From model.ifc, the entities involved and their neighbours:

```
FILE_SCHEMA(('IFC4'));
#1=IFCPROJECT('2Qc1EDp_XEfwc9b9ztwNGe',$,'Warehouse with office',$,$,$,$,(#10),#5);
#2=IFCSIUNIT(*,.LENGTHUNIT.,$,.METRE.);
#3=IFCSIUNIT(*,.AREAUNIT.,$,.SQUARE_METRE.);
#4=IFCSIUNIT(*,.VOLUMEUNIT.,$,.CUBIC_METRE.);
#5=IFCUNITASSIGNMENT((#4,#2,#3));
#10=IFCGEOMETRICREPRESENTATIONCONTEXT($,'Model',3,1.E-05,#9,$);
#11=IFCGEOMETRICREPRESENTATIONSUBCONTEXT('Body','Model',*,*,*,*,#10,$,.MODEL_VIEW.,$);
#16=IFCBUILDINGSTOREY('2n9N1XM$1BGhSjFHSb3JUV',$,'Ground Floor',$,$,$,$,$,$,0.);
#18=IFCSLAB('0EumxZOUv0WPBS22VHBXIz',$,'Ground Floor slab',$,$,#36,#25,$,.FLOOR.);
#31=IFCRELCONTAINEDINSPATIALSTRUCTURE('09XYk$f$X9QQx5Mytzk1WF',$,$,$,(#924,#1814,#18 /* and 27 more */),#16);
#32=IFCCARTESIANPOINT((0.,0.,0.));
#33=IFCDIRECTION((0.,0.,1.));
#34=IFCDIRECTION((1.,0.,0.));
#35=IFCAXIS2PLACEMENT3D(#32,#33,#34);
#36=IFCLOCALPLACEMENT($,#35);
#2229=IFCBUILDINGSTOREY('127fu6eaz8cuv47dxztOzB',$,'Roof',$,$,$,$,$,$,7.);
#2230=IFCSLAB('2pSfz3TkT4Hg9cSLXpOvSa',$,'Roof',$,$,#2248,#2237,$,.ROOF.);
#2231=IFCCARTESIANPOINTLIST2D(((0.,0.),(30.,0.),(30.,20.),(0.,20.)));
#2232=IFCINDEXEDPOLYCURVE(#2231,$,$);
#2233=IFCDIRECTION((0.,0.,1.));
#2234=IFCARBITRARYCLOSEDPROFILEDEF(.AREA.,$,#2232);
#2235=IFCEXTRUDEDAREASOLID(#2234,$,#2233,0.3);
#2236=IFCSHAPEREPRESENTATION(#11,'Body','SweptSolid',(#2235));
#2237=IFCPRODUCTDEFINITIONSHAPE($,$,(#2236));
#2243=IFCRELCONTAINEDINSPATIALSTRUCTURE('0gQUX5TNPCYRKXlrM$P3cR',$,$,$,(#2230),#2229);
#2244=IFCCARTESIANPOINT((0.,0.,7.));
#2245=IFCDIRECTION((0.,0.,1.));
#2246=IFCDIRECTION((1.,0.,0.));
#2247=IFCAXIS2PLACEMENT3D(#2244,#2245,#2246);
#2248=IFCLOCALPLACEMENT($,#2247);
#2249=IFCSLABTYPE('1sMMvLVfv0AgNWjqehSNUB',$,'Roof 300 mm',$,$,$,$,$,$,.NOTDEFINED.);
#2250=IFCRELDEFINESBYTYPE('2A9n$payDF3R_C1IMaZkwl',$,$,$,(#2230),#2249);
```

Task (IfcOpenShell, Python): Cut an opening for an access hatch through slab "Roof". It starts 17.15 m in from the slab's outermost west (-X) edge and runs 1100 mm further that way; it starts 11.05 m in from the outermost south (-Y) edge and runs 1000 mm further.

```python
import numpy as np
import ifcopenshell
import ifcopenshell.api.feature
import ifcopenshell.api.geometry
import ifcopenshell.api.root
import ifcopenshell.geom
import ifcopenshell.util.placement
import ifcopenshell.util.representation
import ifcopenshell.util.shape
import ifcopenshell.util.unit

model = ifcopenshell.open("model.ifc")
unit_scale = ifcopenshell.util.unit.calculate_unit_scale(model)
settings = ifcopenshell.geom.settings()


def volume(element):
    """Net volume in cubic metres, openings subtracted."""
    shape = ifcopenshell.geom.create_shape(settings, element)
    return ifcopenshell.util.shape.get_volume(shape.geometry)


slab = model.by_id(2230)
before = volume(slab)

# Extent in the slab's own axes, in metres. The edges named are its -X and -Y sides.
slab_shape = ifcopenshell.geom.create_shape(settings, slab)
vertices = ifcopenshell.util.shape.get_vertices(slab_shape.geometry)
x_min, y_min, bottom = vertices.min(axis=0)
top = vertices[:, 2].max()

opening = ifcopenshell.api.root.create_entity(model, ifc_class="IfcOpeningElement", name="Access hatch opening", predefined_type="OPENING")
context = ifcopenshell.util.representation.get_context(model, "Model", "Body", "MODEL_VIEW")
width, depth = 1.1, 1
outline = [(0.0, 0.0), (width, 0.0), (width, depth), (0.0, depth), (0.0, 0.0)]
# Overshoot both faces by 50 mm so the cut is clean.
shape = ifcopenshell.api.geometry.add_slab_representation(
    model, context=context, depth=top - bottom + 0.1, polyline=outline
)
ifcopenshell.api.geometry.assign_representation(model, product=opening, representation=shape)

matrix = ifcopenshell.util.placement.get_local_placement(slab.ObjectPlacement)
matrix[:, 3] = matrix @ np.append(np.array([x_min + 17.15, y_min + 11.05, bottom - 0.05]) / unit_scale, 1.0)
ifcopenshell.api.geometry.edit_object_placement(model, product=opening, matrix=matrix, is_si=False)
ifcopenshell.api.feature.add_feature(model, feature=opening, element=slab)

after = volume(slab)

print(f"slab volume {before:.3f} -> {after:.3f} m3")

model.write("model_rev.ifc")
```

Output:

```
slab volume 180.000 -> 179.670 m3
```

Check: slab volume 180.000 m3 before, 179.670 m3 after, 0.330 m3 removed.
